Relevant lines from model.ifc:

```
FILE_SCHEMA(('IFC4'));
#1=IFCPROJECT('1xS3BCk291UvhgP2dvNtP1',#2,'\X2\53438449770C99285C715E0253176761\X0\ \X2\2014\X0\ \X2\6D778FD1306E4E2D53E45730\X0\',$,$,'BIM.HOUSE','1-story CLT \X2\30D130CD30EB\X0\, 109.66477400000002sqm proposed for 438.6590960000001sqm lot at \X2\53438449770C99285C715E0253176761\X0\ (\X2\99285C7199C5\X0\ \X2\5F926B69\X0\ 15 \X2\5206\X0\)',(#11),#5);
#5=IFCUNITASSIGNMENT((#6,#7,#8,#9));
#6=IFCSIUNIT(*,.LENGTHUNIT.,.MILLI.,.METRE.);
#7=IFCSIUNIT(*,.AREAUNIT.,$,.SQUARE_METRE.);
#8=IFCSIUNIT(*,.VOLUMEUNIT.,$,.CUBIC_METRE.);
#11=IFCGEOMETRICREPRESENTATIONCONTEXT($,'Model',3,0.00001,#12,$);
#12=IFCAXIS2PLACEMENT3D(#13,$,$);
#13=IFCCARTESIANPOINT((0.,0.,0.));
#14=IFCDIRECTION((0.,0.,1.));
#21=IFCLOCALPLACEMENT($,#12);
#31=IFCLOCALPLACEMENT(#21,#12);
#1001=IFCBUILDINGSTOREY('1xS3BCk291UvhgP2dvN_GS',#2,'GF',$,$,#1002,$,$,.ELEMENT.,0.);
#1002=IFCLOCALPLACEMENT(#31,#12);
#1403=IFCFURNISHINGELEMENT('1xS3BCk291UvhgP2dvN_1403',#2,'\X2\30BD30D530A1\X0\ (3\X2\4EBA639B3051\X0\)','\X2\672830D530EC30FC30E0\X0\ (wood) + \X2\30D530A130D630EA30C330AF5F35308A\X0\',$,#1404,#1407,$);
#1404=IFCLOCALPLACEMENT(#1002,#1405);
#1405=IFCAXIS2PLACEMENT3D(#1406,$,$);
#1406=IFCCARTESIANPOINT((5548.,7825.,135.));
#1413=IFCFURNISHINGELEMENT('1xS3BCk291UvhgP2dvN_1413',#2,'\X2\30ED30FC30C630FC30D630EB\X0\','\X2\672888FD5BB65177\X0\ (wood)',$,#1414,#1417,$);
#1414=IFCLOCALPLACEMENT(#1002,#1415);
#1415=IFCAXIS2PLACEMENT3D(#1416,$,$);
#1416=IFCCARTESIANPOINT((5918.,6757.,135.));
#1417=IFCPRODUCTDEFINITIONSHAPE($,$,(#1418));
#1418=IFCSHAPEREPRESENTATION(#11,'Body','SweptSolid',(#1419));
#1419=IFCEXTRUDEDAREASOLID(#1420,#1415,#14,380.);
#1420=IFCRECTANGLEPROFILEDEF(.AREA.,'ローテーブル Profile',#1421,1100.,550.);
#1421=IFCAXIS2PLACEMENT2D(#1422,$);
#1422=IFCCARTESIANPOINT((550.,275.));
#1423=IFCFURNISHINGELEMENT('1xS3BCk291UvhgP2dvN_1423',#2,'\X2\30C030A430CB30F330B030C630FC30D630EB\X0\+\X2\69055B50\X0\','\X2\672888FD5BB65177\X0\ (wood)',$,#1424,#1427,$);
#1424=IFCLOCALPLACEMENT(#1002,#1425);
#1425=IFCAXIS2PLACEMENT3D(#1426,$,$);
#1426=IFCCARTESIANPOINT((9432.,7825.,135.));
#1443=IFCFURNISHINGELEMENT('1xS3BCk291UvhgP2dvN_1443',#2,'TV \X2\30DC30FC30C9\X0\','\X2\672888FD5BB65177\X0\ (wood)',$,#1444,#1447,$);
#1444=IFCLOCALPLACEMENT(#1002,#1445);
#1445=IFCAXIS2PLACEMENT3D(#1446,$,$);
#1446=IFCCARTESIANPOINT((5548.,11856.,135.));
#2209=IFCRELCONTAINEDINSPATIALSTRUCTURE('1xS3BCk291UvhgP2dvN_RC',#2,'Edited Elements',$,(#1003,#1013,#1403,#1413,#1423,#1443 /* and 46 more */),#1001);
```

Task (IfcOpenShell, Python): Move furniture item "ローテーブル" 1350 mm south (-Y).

```python
import ifcopenshell
import ifcopenshell.api.geometry
import ifcopenshell.util.placement

model = ifcopenshell.open("model.ifc")

item = model.by_guid("1xS3BCk291UvhgP2dvN_1413")
matrix = ifcopenshell.util.placement.get_local_placement(item.ObjectPlacement)
matrix[1, 3] -= 1350.0
ifcopenshell.api.geometry.edit_object_placement(model, product=item, matrix=matrix, is_si=False)

print(ifcopenshell.util.placement.get_local_placement(item.ObjectPlacement).round(3) + 0.0)

model.write("model_edited.ifc")
```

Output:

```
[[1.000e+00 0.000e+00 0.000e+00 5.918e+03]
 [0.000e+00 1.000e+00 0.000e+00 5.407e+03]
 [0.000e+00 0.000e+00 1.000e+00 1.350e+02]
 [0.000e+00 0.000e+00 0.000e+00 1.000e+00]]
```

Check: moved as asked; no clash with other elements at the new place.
